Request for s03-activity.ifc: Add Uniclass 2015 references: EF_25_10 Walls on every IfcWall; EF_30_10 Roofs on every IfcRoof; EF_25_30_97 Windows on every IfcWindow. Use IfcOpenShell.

First a look at what the model holds.

```python
import ifcopenshell

model = ifcopenshell.open("s03-activity.ifc")
print(model.schema)
print("classifications:", [c.Name for c in model.by_type("IfcClassification")])
for ifc_class in ("IfcDoor", "IfcRoof", "IfcStair", "IfcWall", "IfcWindow"):
    print(ifc_class, len(model.by_type(ifc_class)))
```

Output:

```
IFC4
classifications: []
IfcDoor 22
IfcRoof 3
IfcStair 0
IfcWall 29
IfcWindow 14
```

```python
import ifcopenshell
import ifcopenshell.api.classification

model = ifcopenshell.open("s03-activity.ifc")

system = ifcopenshell.api.classification.add_classification(model, classification="Uniclass 2015")

codes = {
    "IfcWall": ("EF_25_10", "Walls"),
    "IfcRoof": ("EF_30_10", "Roofs"),
    "IfcWindow": ("EF_25_30_97", "Windows"),
}
for ifc_class, (code, name) in codes.items():
    products = model.by_type(ifc_class)
    ifcopenshell.api.classification.add_reference(
        model, products=products, classification=system, identification=code, name=name
    )
    print(code, len(products))

model.write("s03-activity_v2.ifc")
```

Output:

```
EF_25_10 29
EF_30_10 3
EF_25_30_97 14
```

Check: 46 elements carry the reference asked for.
